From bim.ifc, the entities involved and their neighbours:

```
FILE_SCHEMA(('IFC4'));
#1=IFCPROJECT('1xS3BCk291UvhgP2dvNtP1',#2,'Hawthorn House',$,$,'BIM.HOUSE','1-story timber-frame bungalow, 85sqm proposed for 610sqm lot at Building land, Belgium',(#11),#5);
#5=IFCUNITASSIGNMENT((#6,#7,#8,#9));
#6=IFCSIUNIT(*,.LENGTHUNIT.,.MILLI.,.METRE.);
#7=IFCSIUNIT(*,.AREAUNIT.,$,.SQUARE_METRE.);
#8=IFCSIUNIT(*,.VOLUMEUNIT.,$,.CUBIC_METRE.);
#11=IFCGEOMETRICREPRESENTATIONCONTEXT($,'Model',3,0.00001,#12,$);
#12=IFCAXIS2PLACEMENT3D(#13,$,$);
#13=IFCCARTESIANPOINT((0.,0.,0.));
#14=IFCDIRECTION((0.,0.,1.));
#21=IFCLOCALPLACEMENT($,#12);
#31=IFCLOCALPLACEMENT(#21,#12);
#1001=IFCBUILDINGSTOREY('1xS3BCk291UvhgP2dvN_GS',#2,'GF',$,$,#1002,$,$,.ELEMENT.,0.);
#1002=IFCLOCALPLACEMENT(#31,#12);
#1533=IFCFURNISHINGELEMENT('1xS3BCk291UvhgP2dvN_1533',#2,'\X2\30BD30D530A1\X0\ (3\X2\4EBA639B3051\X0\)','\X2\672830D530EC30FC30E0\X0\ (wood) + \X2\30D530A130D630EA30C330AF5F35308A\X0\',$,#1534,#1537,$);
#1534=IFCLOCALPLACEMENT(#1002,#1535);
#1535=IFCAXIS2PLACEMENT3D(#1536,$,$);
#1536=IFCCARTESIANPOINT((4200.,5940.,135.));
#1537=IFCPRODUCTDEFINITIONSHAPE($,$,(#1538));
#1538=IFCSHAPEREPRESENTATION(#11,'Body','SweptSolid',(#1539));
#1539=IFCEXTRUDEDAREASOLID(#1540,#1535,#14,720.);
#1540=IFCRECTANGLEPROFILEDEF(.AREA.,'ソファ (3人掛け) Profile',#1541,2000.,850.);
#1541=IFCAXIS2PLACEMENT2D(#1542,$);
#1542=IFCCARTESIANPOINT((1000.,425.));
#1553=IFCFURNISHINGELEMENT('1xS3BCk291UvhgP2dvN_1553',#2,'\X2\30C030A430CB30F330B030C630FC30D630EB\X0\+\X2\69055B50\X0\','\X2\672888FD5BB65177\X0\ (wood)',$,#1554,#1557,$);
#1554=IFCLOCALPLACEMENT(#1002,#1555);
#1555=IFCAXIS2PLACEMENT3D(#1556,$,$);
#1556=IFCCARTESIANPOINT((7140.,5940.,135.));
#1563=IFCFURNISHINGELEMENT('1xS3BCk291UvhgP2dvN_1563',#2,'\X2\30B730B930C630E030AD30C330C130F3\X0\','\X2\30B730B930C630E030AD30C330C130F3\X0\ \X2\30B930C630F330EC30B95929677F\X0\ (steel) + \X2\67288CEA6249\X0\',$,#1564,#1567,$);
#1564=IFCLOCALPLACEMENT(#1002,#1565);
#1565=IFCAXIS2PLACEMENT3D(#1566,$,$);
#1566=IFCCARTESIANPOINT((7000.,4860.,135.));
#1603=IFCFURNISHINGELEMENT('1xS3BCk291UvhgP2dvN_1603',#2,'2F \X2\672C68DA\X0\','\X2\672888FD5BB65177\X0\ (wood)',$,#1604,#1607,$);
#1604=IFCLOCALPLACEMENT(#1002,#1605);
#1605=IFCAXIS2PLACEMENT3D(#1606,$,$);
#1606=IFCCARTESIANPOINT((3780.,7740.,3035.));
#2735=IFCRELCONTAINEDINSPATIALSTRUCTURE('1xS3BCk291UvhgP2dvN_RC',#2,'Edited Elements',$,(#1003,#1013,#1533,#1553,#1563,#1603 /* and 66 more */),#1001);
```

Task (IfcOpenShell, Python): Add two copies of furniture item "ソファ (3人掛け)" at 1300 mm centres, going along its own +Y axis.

```python
import ifcopenshell
import ifcopenshell.api.geometry
import ifcopenshell.api.root
import ifcopenshell.util.element
import ifcopenshell.util.placement
import ifcopenshell.util.unit

model = ifcopenshell.open("bim.ifc")
unit_scale = ifcopenshell.util.unit.calculate_unit_scale(model)


def reuse_history(source, copy):
    """copy_class also copies each property set's owner history, people and application; keep the originals."""
    for rel in copy.IsDefinedBy:
        if rel.is_a("IfcRelDefinesByProperties") and (history := rel.RelatingPropertyDefinition.OwnerHistory):
            rel.RelatingPropertyDefinition.OwnerHistory = source.OwnerHistory
            ifcopenshell.util.element.remove_deep2(model, history)


source = model.by_guid("1xS3BCk291UvhgP2dvN_1533")
base = ifcopenshell.util.placement.get_local_placement(source.ObjectPlacement)
step = base[:3, 1] * 1.3 / unit_scale

for i in range(1, 3):
    copy = ifcopenshell.api.root.copy_class(model, product=source)
    copy.Representation = ifcopenshell.util.element.copy_deep(
        model, source.Representation, exclude=["IfcGeometricRepresentationContext", "IfcRepresentationMap"]
    )
    reuse_history(source, copy)
    matrix = base.copy()
    matrix[:3, 3] += i * step
    print("added at", matrix[:3, 3].round(3) + 0.0)
    ifcopenshell.api.geometry.edit_object_placement(model, product=copy, matrix=matrix, is_si=False)

model.write("bim-out.ifc")
```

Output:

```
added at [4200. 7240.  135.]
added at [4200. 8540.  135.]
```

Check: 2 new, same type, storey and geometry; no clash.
